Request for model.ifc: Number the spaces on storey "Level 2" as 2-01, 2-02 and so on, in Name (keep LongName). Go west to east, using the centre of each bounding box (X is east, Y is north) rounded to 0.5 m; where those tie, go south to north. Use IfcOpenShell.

First a look at what the model holds.

```python
import ifcopenshell
import ifcopenshell.util.element
import ifcopenshell.util.placement

model = ifcopenshell.open("model.ifc")
print(model.schema)
storey = next(s for s in model.by_type("IfcBuildingStorey") if s.Name == "Level 2")
spaces = [e for e in ifcopenshell.util.element.get_decomposition(storey) if e.is_a("IfcSpace")]
for e in sorted(spaces, key=lambda e: e.id()):
    origin = ifcopenshell.util.placement.get_local_placement(e.ObjectPlacement)[:3, 3]
    print(e.id(), e.Name, e.LongName, origin.round(2) + 0.0, sep=" | ")
```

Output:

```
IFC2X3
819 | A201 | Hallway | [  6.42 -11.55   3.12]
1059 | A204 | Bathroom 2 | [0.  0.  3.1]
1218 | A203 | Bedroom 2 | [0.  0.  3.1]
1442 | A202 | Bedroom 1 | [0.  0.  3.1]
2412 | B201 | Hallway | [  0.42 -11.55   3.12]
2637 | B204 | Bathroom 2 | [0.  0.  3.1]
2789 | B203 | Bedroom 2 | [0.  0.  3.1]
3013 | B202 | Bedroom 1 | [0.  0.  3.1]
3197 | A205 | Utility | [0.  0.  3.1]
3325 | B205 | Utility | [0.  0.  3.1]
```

```python
import ifcopenshell
import ifcopenshell.geom
import ifcopenshell.util.element
import ifcopenshell.util.shape

model = ifcopenshell.open("model.ifc")
settings = ifcopenshell.geom.settings()
settings.set("use-world-coords", True)


def centre(element):
    shape = ifcopenshell.geom.create_shape(settings, element)
    return ifcopenshell.util.shape.get_bbox_centroid(shape.geometry)


storey = next(s for s in model.by_type("IfcBuildingStorey") if s.Name == "Level 2")
spaces = [e for e in ifcopenshell.util.element.get_decomposition(storey) if e.is_a("IfcSpace")]

# Insertion points can sit at a corner or the storey origin, so sort by the geometry (in metres).
centres = {e: centre(e) for e in spaces}
spaces.sort(key=lambda e: (round(centres[e][0] / 0.5), centres[e][1]))

for i, e in enumerate(spaces, start=1):
    number = f"2-{i:02d}"
    e.Name = number
    print(e.id(), number)

model.write("model_rev.ifc")
```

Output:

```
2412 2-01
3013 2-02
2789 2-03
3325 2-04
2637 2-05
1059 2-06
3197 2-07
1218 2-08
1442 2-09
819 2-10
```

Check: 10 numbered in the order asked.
